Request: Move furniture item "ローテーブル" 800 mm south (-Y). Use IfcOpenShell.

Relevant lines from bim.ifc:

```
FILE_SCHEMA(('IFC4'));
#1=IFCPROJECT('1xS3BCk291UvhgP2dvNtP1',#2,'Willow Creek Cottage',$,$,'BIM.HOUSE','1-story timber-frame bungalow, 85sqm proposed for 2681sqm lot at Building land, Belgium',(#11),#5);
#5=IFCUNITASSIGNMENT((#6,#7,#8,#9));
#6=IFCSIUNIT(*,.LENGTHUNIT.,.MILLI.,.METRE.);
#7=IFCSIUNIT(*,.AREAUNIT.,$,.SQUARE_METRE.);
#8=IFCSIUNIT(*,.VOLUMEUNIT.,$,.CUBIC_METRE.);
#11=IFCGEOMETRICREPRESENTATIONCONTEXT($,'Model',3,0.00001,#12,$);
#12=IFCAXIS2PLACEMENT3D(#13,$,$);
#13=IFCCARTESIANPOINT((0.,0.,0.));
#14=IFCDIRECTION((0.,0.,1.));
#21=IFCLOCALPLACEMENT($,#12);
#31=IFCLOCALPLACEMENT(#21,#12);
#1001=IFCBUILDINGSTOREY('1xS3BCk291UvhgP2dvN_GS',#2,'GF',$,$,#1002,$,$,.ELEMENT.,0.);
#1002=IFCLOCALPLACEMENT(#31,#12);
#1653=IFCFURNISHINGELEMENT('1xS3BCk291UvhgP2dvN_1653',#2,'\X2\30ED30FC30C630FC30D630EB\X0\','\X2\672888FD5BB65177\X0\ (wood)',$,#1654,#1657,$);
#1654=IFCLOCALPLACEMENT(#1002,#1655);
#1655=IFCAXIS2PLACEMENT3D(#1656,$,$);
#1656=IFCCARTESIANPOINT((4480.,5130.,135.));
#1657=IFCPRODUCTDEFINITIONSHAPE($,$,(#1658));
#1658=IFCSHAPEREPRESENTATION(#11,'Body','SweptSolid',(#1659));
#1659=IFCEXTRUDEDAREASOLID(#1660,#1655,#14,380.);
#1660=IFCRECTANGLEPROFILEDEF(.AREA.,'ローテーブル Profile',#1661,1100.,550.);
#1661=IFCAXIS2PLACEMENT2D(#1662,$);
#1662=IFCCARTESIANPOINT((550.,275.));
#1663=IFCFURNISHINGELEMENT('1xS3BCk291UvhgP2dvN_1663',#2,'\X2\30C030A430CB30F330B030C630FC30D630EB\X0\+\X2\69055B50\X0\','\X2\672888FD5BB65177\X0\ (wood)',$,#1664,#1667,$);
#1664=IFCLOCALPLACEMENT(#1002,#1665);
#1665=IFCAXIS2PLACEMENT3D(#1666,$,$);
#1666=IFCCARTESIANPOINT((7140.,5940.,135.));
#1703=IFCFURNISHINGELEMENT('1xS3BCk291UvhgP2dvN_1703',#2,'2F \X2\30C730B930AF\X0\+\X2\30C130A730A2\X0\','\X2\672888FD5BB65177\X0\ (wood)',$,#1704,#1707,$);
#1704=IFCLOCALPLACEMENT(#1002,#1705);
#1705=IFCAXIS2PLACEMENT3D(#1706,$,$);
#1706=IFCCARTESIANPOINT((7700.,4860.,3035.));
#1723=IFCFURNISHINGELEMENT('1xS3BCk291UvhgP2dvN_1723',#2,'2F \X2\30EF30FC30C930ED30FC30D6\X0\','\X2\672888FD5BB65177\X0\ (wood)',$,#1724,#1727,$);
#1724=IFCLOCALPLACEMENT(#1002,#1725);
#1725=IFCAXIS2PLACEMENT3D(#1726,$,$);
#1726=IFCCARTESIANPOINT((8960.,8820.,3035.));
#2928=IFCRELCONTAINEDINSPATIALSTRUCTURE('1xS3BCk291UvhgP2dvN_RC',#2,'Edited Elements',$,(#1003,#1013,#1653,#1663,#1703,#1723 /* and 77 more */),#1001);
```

```python
import ifcopenshell
import ifcopenshell.api.geometry
import ifcopenshell.util.placement
import ifcopenshell.util.unit

model = ifcopenshell.open("bim.ifc")
unit_scale = ifcopenshell.util.unit.calculate_unit_scale(model)

item = model.by_guid("1xS3BCk291UvhgP2dvN_1653")
matrix = ifcopenshell.util.placement.get_local_placement(item.ObjectPlacement)
matrix[1, 3] -= 0.8 / unit_scale
ifcopenshell.api.geometry.edit_object_placement(model, product=item, matrix=matrix, is_si=False)

print(ifcopenshell.util.placement.get_local_placement(item.ObjectPlacement).round(3) + 0.0)

model.write("bim_v2.ifc")
```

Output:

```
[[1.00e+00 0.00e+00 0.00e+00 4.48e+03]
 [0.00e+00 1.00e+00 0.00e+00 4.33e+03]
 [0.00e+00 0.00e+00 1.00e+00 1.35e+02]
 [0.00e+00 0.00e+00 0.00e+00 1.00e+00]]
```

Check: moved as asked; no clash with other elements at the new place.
